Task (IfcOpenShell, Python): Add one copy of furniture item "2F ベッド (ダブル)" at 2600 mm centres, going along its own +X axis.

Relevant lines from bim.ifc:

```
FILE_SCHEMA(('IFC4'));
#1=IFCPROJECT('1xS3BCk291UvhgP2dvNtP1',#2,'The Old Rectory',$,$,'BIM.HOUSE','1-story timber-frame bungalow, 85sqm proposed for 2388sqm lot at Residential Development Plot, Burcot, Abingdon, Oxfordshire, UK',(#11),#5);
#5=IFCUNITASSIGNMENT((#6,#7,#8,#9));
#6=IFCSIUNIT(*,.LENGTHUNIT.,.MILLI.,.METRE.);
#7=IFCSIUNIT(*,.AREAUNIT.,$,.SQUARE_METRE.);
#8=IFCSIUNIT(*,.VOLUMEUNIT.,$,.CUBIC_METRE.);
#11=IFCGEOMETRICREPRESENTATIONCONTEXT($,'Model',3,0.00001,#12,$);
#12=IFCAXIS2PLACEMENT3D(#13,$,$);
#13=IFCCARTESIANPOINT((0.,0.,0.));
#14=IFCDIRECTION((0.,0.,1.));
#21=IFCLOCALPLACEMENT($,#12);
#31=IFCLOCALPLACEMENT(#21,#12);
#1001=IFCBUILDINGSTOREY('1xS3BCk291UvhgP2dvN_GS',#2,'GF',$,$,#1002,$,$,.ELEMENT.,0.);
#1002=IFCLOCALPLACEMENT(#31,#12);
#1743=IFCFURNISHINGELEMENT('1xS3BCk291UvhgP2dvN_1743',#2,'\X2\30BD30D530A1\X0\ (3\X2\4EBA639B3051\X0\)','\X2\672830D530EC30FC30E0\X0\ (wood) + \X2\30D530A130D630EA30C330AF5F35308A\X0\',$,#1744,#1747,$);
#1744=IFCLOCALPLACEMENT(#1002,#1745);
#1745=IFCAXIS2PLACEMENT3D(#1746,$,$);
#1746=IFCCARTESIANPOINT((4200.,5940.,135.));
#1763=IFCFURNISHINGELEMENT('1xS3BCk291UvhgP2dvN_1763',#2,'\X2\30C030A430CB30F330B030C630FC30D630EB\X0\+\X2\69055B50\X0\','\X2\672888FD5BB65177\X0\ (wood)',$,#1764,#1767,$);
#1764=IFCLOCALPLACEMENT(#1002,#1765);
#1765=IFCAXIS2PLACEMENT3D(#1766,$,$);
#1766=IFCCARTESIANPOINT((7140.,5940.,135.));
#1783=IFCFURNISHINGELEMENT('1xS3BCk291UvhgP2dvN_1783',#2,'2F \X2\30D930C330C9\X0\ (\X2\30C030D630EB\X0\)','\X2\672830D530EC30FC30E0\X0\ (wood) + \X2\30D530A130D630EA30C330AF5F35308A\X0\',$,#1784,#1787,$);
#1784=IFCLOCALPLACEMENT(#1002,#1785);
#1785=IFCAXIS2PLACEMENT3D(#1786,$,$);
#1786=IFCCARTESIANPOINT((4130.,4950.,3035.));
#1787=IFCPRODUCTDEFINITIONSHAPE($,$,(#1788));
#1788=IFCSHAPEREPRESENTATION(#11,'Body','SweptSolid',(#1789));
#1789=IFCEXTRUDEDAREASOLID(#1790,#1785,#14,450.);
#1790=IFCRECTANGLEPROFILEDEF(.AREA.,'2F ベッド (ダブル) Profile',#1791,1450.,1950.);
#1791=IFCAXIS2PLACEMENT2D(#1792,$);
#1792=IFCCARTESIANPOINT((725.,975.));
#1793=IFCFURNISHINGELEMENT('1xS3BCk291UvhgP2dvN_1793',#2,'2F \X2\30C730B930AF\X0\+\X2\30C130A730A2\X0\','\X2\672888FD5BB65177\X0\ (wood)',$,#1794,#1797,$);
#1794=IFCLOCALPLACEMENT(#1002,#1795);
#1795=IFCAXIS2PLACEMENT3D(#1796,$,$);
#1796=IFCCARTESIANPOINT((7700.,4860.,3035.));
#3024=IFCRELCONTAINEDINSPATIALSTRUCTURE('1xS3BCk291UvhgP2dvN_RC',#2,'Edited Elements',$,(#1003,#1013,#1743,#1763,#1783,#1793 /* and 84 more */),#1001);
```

```python
import ifcopenshell
import ifcopenshell.api.geometry
import ifcopenshell.api.root
import ifcopenshell.util.element
import ifcopenshell.util.placement
import ifcopenshell.util.unit

model = ifcopenshell.open("bim.ifc")
unit_scale = ifcopenshell.util.unit.calculate_unit_scale(model)


def reuse_history(source, copy):
    """copy_class also copies each property set's owner history, people and application; keep the originals."""
    for rel in copy.IsDefinedBy:
        if rel.is_a("IfcRelDefinesByProperties") and (history := rel.RelatingPropertyDefinition.OwnerHistory):
            rel.RelatingPropertyDefinition.OwnerHistory = source.OwnerHistory
            ifcopenshell.util.element.remove_deep2(model, history)


source = model.by_guid("1xS3BCk291UvhgP2dvN_1783")
base = ifcopenshell.util.placement.get_local_placement(source.ObjectPlacement)
step = base[:3, 0] * 2.6 / unit_scale

for i in range(1, 2):
    copy = ifcopenshell.api.root.copy_class(model, product=source)
    copy.Representation = ifcopenshell.util.element.copy_deep(
        model, source.Representation, exclude=["IfcGeometricRepresentationContext", "IfcRepresentationMap"]
    )
    reuse_history(source, copy)
    matrix = base.copy()
    matrix[:3, 3] += i * step
    print("added at", matrix[:3, 3].round(3) + 0.0)
    ifcopenshell.api.geometry.edit_object_placement(model, product=copy, matrix=matrix, is_si=False)

model.write("bim-out.ifc")
```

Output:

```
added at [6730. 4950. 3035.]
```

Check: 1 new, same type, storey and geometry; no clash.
